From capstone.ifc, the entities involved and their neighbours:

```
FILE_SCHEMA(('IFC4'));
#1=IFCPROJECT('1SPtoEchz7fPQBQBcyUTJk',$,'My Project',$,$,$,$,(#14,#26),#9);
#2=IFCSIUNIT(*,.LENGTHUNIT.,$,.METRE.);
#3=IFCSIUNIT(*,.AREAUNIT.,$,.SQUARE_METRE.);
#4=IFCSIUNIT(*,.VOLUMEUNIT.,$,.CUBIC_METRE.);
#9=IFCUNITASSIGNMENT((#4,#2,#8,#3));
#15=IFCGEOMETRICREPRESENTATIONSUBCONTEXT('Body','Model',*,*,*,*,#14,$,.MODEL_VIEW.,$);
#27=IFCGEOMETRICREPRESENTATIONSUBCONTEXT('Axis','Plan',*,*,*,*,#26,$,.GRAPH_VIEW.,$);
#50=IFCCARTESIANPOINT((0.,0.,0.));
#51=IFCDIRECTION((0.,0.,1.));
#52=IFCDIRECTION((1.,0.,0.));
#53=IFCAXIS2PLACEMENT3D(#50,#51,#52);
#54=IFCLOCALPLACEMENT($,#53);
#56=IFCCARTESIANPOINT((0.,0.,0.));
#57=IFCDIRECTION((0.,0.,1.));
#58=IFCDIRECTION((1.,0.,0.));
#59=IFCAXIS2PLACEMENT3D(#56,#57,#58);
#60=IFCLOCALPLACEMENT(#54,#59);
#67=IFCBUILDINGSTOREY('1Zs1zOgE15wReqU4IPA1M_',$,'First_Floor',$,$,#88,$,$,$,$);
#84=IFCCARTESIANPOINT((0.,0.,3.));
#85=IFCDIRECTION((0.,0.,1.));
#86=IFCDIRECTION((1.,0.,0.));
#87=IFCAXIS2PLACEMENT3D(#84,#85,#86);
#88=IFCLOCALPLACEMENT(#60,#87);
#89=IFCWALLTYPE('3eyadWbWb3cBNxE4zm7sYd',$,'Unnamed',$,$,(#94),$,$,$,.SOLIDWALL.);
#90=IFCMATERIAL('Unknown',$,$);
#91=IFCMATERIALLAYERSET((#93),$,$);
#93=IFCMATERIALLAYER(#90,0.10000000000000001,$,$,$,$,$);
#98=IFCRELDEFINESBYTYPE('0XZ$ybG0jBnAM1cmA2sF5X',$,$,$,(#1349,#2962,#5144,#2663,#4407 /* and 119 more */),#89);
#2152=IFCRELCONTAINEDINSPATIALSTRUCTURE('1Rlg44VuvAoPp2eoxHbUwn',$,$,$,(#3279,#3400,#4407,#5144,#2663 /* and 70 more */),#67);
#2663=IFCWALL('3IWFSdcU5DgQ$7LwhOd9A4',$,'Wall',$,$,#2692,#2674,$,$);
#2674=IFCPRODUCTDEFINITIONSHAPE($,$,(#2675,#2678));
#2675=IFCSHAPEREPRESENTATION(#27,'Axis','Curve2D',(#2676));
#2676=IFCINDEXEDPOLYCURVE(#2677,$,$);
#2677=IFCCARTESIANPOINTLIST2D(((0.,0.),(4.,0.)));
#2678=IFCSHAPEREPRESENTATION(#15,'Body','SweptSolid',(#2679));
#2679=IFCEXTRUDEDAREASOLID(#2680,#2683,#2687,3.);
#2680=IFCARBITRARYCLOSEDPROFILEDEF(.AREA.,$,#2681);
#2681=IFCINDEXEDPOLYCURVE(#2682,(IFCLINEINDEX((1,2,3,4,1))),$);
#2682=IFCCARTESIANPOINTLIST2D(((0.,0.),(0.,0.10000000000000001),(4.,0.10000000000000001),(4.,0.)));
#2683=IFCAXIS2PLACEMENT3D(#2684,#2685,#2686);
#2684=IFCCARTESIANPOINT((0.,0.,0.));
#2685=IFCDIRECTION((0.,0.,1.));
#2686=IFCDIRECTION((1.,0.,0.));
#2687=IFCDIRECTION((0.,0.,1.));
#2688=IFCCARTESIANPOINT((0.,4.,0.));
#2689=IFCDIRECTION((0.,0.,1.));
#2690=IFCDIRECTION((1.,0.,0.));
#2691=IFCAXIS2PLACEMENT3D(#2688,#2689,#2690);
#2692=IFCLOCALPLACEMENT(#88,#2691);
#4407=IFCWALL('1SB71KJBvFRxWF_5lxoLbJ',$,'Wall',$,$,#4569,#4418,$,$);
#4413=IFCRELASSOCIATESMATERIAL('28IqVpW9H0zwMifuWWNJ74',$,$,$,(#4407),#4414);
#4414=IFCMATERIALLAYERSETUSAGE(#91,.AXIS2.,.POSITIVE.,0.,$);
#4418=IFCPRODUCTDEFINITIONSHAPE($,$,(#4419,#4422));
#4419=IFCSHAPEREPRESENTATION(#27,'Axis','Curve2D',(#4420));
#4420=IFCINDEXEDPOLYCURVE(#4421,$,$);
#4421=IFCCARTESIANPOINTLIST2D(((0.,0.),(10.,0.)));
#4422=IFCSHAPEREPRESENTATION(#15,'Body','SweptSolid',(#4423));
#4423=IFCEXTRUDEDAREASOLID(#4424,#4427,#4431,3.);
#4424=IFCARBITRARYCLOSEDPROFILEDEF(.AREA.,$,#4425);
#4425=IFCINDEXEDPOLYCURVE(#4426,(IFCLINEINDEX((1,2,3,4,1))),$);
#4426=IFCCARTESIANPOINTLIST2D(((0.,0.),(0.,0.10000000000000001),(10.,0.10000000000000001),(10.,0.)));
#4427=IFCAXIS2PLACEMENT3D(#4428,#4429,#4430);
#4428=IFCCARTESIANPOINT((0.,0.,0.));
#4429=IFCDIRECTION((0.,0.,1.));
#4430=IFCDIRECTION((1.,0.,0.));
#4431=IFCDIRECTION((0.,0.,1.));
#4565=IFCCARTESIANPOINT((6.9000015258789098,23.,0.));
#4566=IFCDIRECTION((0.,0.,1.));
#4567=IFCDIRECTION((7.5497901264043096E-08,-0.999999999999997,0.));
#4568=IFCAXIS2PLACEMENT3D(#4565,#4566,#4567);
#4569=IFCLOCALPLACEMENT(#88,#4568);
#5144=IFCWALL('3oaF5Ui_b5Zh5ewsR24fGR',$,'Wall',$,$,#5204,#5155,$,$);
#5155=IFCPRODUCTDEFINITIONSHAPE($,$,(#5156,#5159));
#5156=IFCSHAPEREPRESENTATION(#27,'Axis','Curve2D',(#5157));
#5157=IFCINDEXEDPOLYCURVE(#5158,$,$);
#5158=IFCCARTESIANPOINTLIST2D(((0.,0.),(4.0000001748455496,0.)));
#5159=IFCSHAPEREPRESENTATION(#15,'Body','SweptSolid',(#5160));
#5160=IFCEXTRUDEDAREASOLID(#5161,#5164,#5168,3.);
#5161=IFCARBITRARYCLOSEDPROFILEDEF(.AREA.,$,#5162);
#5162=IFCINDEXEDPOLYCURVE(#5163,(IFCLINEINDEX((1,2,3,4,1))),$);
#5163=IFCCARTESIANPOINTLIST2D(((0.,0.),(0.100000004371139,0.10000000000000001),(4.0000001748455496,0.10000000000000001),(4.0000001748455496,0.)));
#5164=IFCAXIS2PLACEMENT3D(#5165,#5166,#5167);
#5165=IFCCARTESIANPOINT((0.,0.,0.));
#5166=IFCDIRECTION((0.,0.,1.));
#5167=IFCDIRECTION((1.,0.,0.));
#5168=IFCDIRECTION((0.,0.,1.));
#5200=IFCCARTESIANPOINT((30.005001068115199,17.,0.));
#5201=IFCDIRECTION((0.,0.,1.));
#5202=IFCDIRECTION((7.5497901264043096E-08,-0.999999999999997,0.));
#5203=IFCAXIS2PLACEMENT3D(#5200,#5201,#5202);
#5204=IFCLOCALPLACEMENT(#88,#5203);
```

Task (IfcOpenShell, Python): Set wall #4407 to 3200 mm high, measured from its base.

```python
import ifcopenshell
import ifcopenshell.geom
import ifcopenshell.util.representation
import ifcopenshell.util.shape
import ifcopenshell.util.unit

model = ifcopenshell.open("capstone.ifc")
unit_scale = ifcopenshell.util.unit.calculate_unit_scale(model)
settings = ifcopenshell.geom.settings()


def volume(element):
    """Net volume in cubic metres, openings subtracted."""
    shape = ifcopenshell.geom.create_shape(settings, element)
    return ifcopenshell.util.shape.get_volume(shape.geometry)


wall = model.by_guid("1SB71KJBvFRxWF_5lxoLbJ")
before = volume(wall)

body = ifcopenshell.util.representation.get_representation(wall, "Model", "Body")
solid = body.Items[0]
old_height = solid.Depth
solid.Depth = 3.2 / unit_scale
after = volume(wall)

print(f"height {old_height:g} -> {solid.Depth:g}, volume {before:.3f} -> {after:.3f} m3")

model.write("capstone-out.ifc")
```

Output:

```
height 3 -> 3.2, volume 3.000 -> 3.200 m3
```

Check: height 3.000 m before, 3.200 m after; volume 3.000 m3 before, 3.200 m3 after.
